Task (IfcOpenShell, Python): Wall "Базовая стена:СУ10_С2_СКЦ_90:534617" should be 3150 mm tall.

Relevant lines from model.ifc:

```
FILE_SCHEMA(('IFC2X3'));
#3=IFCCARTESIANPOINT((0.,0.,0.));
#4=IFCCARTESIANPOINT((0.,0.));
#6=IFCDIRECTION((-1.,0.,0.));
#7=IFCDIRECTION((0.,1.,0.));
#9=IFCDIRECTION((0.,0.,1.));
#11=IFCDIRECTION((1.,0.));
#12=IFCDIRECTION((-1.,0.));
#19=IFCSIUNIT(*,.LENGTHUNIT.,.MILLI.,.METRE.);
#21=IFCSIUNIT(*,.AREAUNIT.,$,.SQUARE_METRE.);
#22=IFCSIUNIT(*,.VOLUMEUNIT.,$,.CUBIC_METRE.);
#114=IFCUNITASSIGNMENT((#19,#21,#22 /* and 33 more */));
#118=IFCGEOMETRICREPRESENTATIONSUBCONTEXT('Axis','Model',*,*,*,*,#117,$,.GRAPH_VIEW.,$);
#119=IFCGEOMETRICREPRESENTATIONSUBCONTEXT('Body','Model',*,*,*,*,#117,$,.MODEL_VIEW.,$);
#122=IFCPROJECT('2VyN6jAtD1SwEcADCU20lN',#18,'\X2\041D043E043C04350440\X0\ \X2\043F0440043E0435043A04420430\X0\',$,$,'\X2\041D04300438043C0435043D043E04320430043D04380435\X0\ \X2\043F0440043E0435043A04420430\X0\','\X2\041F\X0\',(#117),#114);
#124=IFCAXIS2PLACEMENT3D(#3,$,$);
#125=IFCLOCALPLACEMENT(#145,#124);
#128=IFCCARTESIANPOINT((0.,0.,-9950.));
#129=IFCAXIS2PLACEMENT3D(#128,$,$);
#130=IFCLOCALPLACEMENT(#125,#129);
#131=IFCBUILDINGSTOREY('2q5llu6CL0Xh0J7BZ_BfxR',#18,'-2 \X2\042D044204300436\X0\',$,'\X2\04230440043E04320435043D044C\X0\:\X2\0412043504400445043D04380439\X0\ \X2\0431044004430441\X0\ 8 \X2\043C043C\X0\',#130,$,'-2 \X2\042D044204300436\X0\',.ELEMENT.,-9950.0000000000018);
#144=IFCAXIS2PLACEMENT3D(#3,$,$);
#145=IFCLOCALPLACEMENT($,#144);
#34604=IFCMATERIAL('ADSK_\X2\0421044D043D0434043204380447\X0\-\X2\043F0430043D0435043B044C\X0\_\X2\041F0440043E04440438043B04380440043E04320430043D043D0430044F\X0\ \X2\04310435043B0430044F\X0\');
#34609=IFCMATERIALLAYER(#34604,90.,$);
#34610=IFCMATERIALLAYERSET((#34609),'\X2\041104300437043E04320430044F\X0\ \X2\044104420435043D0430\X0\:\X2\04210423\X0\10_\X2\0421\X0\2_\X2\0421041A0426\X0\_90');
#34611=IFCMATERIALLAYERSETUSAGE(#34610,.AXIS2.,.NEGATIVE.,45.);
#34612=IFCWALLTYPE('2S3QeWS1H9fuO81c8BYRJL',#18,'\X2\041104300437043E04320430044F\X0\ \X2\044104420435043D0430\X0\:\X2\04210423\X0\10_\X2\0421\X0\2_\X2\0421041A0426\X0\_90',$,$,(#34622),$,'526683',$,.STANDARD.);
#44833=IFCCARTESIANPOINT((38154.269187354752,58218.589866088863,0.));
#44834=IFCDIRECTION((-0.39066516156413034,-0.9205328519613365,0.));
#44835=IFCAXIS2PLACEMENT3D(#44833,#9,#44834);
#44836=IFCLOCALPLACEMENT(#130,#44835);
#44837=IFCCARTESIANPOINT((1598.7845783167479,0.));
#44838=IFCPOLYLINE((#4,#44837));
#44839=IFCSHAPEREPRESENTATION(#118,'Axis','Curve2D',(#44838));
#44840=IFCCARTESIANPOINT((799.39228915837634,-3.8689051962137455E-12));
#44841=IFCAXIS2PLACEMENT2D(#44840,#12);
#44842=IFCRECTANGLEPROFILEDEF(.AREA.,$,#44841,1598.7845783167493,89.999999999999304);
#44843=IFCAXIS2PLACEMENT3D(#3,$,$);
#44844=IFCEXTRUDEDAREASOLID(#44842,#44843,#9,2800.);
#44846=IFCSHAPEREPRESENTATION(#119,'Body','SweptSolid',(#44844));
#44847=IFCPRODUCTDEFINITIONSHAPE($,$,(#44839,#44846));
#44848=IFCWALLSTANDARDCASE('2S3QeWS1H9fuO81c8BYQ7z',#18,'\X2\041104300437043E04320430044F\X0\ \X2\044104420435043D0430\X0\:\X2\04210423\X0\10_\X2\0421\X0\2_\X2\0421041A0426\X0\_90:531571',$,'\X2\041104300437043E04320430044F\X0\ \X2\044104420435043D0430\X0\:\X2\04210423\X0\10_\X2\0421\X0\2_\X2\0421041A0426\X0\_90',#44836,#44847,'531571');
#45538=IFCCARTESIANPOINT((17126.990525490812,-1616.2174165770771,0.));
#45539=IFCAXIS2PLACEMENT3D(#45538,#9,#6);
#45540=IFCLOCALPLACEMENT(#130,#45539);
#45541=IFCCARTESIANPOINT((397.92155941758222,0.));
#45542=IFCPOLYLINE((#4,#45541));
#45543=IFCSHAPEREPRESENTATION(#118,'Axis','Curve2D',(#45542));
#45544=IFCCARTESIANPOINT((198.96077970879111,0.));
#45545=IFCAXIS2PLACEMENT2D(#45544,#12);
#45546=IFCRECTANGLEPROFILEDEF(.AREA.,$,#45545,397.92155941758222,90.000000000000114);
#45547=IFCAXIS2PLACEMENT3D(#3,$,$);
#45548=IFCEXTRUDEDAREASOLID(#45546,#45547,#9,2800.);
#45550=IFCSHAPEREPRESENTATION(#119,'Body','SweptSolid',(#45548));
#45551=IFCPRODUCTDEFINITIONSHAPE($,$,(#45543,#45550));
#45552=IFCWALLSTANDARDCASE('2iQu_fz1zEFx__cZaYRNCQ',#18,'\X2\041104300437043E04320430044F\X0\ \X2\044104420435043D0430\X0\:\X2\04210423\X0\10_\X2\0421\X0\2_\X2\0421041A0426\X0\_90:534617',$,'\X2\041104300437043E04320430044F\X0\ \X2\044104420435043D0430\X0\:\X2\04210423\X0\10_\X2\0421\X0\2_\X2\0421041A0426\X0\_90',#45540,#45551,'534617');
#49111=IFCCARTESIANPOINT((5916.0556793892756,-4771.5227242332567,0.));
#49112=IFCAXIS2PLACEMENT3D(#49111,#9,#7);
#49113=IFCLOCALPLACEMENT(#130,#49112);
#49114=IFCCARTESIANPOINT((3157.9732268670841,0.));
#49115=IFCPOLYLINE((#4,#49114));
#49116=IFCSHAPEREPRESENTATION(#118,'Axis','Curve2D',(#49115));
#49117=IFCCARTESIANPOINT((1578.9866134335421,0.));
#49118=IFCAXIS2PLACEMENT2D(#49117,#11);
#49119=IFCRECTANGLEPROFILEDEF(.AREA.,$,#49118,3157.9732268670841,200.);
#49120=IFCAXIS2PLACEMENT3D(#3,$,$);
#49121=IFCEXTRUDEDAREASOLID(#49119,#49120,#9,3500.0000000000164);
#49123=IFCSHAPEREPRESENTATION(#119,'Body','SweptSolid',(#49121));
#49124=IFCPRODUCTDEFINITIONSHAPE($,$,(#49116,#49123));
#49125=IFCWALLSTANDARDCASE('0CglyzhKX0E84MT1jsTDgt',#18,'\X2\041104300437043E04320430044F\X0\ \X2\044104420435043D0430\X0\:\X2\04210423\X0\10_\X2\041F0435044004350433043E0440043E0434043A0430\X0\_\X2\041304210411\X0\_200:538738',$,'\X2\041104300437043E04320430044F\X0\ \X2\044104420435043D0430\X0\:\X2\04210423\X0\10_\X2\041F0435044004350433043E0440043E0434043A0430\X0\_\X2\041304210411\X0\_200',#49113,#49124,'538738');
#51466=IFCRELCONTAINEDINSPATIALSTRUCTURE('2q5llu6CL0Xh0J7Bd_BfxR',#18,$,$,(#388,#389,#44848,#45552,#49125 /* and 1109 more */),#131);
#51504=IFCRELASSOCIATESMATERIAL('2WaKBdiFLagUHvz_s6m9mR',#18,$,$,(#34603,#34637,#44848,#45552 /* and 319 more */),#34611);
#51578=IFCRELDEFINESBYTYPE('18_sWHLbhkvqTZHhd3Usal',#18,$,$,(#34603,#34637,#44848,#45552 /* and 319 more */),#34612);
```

```python
import ifcopenshell
import ifcopenshell.geom
import ifcopenshell.util.representation
import ifcopenshell.util.shape
import ifcopenshell.util.unit

model = ifcopenshell.open("model.ifc")
unit_scale = ifcopenshell.util.unit.calculate_unit_scale(model)
settings = ifcopenshell.geom.settings()


def volume(element):
    """Net volume in cubic metres, openings subtracted."""
    shape = ifcopenshell.geom.create_shape(settings, element)
    return ifcopenshell.util.shape.get_volume(shape.geometry)


wall = model.by_id(45552)
before = volume(wall)

body = ifcopenshell.util.representation.get_representation(wall, "Model", "Body")
solid = body.Items[0]
old_height = solid.Depth
solid.Depth = 3.15 / unit_scale
after = volume(wall)

print(f"height {old_height:g} -> {solid.Depth:g}, volume {before:.3f} -> {after:.3f} m3")

model.write("model_v2.ifc")
```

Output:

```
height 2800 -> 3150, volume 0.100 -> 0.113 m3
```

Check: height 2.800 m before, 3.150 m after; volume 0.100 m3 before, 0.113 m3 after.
